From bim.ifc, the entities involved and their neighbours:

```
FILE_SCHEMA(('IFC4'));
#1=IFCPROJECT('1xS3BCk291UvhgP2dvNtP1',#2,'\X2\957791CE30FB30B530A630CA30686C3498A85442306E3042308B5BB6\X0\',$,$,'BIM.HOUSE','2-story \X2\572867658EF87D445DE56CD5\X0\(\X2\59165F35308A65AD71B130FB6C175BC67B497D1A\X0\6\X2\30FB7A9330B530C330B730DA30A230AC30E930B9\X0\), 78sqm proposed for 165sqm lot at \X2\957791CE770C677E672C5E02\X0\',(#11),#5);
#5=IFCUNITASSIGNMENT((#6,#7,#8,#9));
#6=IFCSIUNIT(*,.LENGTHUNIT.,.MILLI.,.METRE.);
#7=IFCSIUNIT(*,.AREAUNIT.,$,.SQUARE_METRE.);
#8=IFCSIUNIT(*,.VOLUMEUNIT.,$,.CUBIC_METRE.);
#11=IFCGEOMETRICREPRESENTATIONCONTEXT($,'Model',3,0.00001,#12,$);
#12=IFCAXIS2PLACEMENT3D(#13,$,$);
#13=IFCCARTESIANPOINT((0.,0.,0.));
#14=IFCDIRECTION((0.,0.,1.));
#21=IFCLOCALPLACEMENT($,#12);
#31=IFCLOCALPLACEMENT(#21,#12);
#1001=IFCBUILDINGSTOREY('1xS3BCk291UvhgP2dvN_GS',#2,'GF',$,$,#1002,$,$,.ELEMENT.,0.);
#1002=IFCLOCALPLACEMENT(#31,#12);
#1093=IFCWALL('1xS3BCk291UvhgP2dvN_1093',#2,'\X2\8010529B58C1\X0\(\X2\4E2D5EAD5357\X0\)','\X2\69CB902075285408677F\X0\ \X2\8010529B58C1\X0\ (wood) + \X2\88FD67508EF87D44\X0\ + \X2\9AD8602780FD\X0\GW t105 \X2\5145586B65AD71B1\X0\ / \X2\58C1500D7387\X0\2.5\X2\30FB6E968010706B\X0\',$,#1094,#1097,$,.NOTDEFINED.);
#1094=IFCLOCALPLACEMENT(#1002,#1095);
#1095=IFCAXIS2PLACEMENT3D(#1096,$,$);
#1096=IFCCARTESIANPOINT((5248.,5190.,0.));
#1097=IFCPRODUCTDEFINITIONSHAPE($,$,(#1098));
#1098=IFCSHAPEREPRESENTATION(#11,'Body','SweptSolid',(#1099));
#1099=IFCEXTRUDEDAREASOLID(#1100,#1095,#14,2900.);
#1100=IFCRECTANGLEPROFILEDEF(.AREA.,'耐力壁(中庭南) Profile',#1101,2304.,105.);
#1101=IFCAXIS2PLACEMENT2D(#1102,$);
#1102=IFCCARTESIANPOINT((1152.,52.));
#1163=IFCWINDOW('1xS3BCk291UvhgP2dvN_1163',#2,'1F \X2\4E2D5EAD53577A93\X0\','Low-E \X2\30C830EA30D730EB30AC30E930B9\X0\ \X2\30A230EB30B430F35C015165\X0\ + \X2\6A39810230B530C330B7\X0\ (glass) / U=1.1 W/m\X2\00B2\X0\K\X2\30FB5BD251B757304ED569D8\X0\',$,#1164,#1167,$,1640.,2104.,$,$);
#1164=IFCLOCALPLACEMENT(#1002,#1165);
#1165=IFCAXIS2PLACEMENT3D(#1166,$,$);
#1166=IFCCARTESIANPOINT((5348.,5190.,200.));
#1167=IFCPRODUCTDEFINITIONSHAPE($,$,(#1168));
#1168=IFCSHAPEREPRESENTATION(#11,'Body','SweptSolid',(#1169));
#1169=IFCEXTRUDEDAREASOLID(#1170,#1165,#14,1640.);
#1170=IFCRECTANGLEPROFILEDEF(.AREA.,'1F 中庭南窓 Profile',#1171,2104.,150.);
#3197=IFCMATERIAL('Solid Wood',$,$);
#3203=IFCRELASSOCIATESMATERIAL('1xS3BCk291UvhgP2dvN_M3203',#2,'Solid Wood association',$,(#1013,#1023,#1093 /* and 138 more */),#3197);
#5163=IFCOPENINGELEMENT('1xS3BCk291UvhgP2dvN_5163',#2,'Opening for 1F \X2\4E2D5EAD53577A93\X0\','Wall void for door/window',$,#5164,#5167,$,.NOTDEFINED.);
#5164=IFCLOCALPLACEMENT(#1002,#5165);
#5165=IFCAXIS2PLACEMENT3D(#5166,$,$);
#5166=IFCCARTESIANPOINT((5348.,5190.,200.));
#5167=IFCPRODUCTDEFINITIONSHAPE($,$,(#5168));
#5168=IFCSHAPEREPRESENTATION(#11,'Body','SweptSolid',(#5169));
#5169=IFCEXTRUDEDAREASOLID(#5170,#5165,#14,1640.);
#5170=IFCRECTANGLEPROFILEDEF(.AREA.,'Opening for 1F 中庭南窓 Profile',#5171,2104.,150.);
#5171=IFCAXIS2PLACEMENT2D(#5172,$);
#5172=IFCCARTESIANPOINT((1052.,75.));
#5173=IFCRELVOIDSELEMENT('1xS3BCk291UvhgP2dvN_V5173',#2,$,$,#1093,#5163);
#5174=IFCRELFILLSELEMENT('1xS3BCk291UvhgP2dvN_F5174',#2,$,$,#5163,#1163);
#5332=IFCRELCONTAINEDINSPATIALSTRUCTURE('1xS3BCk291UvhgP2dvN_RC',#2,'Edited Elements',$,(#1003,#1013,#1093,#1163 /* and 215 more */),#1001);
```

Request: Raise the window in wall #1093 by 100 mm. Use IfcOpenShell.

```python
import numpy as np
import ifcopenshell
import ifcopenshell.api.geometry
import ifcopenshell.util.placement
import ifcopenshell.util.unit

model = ifcopenshell.open("bim.ifc")
unit_scale = ifcopenshell.util.unit.calculate_unit_scale(model)

window = model.by_id(1163)
opening = window.FillsVoids[0].RelatingOpeningElement
dz = 100.0

shift = np.array([0.0, 0.0, dz])
# The window is not placed relative to its opening, so move both.
for product in (opening, window):
    matrix = ifcopenshell.util.placement.get_local_placement(product.ObjectPlacement)
    matrix[:3, 3] += shift
    ifcopenshell.api.geometry.edit_object_placement(model, product=product, matrix=matrix, is_si=False)

print(f"moved by {dz * unit_scale:+.3f} m")

model.write("bim_v2.ifc")
```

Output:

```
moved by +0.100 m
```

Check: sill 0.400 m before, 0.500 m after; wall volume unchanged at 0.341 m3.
